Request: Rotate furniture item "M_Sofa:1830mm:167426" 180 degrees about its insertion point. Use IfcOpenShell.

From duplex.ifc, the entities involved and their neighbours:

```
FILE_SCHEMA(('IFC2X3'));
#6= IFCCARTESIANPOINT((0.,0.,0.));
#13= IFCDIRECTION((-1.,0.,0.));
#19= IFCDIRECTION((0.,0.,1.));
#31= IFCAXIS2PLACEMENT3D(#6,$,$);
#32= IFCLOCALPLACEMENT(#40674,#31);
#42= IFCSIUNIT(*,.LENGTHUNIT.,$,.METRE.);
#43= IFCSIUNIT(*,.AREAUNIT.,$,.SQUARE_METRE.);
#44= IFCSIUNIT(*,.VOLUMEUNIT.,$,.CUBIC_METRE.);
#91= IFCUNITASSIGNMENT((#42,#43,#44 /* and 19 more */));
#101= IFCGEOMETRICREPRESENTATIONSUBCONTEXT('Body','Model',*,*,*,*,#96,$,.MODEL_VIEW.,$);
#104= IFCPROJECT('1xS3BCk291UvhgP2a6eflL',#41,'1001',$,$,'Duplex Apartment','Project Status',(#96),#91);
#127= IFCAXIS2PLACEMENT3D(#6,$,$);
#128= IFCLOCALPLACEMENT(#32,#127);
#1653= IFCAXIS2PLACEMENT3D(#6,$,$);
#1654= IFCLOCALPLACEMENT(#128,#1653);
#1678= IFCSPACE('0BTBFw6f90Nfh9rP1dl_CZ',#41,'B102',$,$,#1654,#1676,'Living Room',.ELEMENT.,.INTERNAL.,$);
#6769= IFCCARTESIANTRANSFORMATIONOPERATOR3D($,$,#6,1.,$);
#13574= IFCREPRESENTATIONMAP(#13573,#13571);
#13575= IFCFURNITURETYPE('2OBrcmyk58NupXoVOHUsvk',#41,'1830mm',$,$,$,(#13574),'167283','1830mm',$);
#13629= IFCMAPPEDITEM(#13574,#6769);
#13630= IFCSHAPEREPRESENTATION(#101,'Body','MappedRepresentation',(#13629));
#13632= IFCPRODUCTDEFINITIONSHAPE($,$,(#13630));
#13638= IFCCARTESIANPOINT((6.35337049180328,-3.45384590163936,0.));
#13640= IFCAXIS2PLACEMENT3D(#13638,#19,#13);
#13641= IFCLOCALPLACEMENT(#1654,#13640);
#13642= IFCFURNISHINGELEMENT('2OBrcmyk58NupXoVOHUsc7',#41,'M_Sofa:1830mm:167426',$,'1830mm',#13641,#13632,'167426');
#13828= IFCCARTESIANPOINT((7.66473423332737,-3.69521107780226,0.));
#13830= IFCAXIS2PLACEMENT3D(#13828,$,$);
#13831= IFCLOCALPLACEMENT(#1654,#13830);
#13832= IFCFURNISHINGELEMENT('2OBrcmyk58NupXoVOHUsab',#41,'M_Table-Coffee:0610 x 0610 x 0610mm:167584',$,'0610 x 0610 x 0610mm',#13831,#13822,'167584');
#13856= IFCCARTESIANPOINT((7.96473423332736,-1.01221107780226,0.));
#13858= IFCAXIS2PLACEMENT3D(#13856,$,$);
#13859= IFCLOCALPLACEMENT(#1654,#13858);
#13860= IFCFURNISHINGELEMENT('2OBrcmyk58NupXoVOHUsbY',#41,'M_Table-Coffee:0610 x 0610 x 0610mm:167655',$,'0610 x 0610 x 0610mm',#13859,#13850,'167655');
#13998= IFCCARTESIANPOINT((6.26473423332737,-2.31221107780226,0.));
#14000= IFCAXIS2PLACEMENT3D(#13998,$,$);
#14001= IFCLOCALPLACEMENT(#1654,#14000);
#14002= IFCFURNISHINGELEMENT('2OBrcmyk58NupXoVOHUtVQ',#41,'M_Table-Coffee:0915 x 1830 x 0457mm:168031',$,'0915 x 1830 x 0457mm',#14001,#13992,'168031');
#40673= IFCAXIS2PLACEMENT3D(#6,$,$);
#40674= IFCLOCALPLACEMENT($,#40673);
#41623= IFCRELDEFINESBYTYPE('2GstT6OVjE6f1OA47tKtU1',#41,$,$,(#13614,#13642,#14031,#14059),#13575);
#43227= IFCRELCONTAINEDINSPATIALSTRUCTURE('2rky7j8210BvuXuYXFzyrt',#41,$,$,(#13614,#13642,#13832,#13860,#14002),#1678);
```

```python
import ifcopenshell
import ifcopenshell.api.geometry
import ifcopenshell.util.placement

model = ifcopenshell.open("duplex.ifc")

item = model.by_guid("2OBrcmyk58NupXoVOHUsc7")
matrix = ifcopenshell.util.placement.get_local_placement(item.ObjectPlacement)
matrix = matrix @ ifcopenshell.util.placement.rotation(180, "Z")
ifcopenshell.api.geometry.edit_object_placement(model, product=item, matrix=matrix, is_si=False)

print(ifcopenshell.util.placement.get_local_placement(item.ObjectPlacement).round(3) + 0.0)

model.write("duplex_updated.ifc")
```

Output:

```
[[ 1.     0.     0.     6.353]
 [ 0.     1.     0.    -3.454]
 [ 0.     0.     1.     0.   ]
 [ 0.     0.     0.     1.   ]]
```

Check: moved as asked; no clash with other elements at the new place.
